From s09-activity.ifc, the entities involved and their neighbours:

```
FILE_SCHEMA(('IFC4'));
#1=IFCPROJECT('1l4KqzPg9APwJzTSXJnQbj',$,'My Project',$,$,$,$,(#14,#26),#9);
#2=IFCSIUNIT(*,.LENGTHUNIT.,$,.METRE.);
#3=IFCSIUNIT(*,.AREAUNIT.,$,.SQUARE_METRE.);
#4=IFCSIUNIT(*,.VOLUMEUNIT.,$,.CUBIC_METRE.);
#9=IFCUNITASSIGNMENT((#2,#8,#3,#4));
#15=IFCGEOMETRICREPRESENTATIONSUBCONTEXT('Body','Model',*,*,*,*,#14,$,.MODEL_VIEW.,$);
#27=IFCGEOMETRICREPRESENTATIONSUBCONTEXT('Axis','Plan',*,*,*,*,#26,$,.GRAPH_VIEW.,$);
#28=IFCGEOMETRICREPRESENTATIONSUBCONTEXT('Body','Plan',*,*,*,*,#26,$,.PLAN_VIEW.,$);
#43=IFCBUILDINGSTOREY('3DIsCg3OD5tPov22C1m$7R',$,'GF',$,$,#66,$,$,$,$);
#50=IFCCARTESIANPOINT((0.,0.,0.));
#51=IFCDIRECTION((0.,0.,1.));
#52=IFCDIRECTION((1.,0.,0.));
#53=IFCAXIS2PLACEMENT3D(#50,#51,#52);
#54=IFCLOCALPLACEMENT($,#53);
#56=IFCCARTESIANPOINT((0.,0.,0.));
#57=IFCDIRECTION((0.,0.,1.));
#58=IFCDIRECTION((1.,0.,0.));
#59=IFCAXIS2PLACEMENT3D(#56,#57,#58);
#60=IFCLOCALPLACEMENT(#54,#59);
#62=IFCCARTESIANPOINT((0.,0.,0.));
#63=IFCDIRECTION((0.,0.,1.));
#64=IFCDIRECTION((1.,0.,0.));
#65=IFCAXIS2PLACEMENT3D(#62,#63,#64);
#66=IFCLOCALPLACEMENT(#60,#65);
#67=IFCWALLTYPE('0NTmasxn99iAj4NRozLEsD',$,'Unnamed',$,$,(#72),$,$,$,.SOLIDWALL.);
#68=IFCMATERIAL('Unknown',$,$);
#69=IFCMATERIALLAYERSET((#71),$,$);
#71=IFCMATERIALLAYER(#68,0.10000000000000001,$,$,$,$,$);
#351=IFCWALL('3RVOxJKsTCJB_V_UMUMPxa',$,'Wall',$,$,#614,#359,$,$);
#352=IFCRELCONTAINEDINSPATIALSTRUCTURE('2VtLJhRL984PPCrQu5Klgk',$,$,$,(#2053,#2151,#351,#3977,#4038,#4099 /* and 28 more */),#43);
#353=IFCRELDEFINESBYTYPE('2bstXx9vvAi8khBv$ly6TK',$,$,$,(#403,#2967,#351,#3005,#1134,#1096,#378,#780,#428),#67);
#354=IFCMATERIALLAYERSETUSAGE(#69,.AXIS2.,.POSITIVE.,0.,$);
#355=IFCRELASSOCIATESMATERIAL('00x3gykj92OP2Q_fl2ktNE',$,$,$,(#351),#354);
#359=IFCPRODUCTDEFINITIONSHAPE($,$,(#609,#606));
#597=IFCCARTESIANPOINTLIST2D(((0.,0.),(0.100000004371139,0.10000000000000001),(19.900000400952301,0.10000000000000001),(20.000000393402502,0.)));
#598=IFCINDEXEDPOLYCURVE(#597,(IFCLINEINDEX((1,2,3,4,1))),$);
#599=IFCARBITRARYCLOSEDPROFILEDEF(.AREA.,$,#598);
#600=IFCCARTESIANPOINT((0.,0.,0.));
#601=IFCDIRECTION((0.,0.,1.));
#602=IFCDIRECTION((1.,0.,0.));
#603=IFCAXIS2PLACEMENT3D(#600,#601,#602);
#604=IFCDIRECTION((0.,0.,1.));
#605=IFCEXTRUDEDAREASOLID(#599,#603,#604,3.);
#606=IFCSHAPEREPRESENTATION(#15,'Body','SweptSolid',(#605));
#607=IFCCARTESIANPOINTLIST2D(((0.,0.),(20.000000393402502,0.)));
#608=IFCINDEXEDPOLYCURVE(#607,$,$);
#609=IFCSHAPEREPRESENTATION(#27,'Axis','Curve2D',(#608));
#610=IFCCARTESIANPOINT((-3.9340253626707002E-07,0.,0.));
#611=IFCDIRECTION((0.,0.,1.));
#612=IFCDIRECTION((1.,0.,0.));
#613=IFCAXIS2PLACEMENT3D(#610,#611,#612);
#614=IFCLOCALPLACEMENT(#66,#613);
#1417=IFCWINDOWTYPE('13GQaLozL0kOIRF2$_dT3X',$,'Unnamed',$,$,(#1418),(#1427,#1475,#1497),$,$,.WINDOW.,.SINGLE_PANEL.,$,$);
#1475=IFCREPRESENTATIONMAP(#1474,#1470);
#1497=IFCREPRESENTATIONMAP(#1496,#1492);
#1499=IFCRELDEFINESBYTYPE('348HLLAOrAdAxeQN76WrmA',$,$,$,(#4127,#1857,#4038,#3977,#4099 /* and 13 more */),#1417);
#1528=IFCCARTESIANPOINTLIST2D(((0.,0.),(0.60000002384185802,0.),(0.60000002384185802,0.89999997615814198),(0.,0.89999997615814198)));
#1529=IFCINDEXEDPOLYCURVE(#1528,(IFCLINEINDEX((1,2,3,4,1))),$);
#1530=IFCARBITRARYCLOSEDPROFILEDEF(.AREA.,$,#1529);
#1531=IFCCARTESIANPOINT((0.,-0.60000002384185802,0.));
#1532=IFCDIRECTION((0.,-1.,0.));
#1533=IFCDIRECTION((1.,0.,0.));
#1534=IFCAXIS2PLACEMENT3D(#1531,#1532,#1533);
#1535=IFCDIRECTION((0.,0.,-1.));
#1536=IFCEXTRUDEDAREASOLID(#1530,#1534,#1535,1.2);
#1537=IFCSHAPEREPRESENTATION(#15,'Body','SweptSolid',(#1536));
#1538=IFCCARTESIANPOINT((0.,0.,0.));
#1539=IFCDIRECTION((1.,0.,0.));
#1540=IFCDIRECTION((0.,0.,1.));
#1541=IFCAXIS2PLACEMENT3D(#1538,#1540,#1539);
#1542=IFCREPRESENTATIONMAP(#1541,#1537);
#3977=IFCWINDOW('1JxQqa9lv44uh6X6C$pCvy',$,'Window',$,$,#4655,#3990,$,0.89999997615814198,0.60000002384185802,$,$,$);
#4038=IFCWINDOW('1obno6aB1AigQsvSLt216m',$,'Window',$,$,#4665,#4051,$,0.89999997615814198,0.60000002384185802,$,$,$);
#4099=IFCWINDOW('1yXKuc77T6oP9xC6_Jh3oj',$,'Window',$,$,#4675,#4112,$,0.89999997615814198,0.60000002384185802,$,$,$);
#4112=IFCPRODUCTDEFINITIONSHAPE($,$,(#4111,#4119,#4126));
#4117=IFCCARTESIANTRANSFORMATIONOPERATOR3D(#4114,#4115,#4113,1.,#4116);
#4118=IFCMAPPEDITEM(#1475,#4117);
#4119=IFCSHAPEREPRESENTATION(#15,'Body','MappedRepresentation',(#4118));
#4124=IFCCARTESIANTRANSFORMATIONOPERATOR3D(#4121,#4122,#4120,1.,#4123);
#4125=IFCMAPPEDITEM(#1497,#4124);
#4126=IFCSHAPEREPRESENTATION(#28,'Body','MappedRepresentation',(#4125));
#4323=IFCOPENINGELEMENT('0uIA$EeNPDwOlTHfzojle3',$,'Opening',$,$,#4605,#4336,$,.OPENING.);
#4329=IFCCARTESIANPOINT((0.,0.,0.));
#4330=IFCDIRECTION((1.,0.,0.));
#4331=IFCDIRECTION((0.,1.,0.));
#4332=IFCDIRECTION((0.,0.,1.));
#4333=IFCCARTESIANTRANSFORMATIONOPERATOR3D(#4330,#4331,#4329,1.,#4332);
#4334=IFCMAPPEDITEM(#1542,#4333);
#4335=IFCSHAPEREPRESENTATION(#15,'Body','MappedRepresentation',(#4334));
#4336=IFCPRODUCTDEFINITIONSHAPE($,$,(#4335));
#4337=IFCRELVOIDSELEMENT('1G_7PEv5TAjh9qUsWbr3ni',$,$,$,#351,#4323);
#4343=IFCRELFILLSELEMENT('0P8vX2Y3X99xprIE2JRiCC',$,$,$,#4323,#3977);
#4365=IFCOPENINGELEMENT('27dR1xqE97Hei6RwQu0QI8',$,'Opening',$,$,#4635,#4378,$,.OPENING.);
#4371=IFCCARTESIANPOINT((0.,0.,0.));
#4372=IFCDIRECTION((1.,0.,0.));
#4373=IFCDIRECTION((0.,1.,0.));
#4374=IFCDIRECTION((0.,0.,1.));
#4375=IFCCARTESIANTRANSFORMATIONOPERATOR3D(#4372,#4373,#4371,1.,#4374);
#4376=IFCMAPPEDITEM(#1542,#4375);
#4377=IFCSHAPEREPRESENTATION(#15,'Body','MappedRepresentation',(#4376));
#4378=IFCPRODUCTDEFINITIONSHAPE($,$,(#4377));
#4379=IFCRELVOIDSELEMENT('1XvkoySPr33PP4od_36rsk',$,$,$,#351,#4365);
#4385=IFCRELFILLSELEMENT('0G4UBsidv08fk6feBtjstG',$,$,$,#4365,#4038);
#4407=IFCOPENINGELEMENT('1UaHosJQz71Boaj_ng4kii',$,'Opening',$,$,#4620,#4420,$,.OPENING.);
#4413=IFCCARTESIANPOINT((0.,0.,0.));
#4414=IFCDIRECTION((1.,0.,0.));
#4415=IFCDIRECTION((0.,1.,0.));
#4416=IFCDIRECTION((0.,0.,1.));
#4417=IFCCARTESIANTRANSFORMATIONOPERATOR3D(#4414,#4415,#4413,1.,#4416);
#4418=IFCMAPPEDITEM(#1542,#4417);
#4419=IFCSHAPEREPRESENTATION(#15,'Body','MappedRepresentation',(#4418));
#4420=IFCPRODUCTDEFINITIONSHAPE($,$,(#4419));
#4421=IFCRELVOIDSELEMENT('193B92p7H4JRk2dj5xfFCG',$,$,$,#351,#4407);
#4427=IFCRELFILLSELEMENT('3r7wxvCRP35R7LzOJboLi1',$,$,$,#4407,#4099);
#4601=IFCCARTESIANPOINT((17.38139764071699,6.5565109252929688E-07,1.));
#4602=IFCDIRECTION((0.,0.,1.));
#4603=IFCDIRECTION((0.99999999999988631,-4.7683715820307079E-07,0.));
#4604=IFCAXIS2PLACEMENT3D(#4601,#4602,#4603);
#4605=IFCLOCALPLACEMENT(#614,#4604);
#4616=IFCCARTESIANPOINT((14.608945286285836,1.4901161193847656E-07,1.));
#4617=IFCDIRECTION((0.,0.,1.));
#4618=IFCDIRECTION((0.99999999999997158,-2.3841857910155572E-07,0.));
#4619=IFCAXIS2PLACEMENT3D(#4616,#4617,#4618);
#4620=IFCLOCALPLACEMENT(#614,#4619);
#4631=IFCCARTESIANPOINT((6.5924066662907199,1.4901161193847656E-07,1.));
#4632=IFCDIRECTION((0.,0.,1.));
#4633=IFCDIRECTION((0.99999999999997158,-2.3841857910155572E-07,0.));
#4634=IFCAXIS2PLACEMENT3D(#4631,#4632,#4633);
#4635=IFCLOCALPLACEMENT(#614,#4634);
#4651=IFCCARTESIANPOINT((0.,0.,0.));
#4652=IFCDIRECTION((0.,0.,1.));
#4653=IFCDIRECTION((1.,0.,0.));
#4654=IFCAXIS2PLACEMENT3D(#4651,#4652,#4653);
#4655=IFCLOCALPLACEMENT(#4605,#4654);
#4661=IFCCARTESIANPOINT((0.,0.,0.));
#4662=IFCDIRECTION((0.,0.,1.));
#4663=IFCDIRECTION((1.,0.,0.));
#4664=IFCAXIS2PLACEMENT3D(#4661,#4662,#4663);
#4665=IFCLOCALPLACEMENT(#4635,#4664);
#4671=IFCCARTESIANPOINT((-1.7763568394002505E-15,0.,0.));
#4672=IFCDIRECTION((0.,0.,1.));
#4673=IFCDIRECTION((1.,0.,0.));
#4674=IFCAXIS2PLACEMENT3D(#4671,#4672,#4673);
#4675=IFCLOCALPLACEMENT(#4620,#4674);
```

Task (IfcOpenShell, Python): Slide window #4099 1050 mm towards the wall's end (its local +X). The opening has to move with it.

```python
import ifcopenshell
import ifcopenshell.api.geometry
import ifcopenshell.util.placement

model = ifcopenshell.open("s09-activity.ifc")

window = model.by_guid("1yXKuc77T6oP9xC6_Jh3oj")
opening = window.FillsVoids[0].RelatingOpeningElement
wall = opening.VoidsElements[0].RelatingBuildingElement

wall_matrix = ifcopenshell.util.placement.get_local_placement(wall.ObjectPlacement)
shift = wall_matrix[:3, 0] * 1.05
before = ifcopenshell.util.placement.get_local_placement(window.ObjectPlacement)[:3, 3].copy()

# The window is placed relative to its opening, so it follows when the opening moves.
matrix = ifcopenshell.util.placement.get_local_placement(opening.ObjectPlacement)
matrix[:3, 3] += shift
ifcopenshell.api.geometry.edit_object_placement(
    model, product=opening, matrix=matrix, is_si=False, should_transform_children=True
)

after = ifcopenshell.util.placement.get_local_placement(window.ObjectPlacement)[:3, 3]
print("window moved by", (after - before).round(3) + 0.0)

model.write("s09-activity_updated.ifc")
```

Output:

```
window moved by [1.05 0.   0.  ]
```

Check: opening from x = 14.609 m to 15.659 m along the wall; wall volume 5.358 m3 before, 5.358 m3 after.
